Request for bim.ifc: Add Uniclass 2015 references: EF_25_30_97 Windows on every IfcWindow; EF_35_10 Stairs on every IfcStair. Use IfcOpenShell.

First a look at what the model holds.

```python
import ifcopenshell

model = ifcopenshell.open("bim.ifc")
print(model.schema)
print("classifications:", [c.Name for c in model.by_type("IfcClassification")])
for ifc_class in ("IfcDoor", "IfcRoof", "IfcStair", "IfcWall", "IfcWindow"):
    print(ifc_class, len(model.by_type(ifc_class)))
```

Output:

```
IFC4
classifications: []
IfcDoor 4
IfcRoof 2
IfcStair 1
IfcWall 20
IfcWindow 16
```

```python
import ifcopenshell
import ifcopenshell.api.classification

model = ifcopenshell.open("bim.ifc")

system = ifcopenshell.api.classification.add_classification(model, classification="Uniclass 2015")

codes = {
    "IfcWindow": ("EF_25_30_97", "Windows"),
    "IfcStair": ("EF_35_10", "Stairs"),
}
for ifc_class, (code, name) in codes.items():
    products = model.by_type(ifc_class)
    ifcopenshell.api.classification.add_reference(
        model, products=products, classification=system, identification=code, name=name
    )
    print(code, len(products))

model.write("bim_v2.ifc")
```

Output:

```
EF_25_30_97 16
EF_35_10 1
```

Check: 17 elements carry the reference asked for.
